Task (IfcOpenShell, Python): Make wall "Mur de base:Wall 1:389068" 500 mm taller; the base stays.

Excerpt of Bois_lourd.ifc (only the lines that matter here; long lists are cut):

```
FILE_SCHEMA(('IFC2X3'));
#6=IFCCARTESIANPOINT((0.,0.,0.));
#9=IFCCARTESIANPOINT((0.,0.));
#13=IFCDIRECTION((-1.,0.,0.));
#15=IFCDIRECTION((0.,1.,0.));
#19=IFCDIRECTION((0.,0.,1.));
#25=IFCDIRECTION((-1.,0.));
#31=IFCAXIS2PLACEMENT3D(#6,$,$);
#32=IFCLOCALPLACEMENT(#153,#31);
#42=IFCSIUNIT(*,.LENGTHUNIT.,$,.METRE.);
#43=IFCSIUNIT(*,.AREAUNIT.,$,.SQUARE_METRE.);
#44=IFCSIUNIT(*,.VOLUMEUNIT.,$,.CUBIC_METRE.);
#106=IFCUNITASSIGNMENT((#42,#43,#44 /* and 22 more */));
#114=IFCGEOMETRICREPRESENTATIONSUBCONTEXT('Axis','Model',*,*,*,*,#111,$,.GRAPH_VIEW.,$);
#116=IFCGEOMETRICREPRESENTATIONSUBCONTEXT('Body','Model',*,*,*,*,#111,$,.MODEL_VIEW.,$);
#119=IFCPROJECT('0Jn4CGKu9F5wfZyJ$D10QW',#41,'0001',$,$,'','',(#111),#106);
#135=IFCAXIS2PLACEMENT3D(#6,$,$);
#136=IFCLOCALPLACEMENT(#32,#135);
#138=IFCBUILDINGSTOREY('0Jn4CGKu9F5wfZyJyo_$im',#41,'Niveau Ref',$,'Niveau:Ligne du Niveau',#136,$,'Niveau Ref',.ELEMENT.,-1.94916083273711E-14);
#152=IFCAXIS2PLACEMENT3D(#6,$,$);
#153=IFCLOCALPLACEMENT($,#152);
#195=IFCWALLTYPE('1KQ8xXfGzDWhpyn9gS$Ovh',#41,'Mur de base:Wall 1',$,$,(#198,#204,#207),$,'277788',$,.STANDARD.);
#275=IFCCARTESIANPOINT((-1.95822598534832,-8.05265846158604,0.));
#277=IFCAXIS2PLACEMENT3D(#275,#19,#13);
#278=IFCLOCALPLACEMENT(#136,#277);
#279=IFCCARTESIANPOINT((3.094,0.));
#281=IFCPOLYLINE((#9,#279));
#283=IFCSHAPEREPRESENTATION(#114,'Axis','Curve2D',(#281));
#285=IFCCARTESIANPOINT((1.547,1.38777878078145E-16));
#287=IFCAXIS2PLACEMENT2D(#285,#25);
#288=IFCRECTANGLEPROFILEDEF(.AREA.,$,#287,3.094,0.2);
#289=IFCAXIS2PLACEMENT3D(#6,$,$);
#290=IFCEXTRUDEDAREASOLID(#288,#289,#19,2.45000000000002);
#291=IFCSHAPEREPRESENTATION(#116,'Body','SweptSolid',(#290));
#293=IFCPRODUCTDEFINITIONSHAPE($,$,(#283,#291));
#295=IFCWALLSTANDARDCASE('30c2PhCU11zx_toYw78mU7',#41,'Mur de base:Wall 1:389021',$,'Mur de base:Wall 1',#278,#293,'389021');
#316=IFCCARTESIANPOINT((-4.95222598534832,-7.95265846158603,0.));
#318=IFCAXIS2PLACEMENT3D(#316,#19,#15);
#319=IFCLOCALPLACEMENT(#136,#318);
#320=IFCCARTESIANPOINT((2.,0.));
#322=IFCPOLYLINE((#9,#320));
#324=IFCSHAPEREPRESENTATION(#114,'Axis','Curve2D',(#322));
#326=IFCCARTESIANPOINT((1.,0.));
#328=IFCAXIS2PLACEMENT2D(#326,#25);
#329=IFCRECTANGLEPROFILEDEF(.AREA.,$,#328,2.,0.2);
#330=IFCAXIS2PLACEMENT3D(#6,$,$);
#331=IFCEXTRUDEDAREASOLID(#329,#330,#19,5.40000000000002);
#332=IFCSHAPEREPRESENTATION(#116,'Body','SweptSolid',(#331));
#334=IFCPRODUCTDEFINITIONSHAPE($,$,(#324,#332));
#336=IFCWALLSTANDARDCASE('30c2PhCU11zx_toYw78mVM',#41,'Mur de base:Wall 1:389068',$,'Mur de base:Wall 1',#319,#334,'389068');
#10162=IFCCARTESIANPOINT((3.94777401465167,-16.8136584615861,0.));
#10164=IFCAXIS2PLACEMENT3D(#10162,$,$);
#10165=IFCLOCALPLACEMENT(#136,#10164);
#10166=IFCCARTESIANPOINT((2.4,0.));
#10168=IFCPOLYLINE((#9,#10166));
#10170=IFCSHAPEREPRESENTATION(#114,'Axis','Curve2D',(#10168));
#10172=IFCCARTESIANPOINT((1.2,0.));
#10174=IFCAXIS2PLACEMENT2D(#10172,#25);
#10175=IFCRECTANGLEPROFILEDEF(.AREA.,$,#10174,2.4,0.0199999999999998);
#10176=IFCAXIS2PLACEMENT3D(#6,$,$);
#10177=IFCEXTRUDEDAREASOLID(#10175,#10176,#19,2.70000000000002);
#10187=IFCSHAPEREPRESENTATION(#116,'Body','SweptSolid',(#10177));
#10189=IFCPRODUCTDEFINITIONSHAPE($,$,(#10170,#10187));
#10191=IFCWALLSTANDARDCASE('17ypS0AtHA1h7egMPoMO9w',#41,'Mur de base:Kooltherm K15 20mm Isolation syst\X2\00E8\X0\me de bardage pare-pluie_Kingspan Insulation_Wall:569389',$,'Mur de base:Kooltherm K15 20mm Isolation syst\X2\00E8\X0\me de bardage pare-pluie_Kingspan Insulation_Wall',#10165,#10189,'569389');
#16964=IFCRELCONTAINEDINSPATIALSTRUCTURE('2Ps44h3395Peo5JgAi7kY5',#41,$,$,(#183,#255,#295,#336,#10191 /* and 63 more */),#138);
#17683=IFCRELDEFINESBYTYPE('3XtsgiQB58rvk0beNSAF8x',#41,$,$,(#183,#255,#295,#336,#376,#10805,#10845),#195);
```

```python
import ifcopenshell
import ifcopenshell.geom
import ifcopenshell.util.representation
import ifcopenshell.util.shape
import ifcopenshell.util.unit

model = ifcopenshell.open("Bois_lourd.ifc")
unit_scale = ifcopenshell.util.unit.calculate_unit_scale(model)
settings = ifcopenshell.geom.settings()


def volume(element):
    """Net volume in cubic metres, openings subtracted."""
    shape = ifcopenshell.geom.create_shape(settings, element)
    return ifcopenshell.util.shape.get_volume(shape.geometry)


wall = model.by_guid("30c2PhCU11zx_toYw78mVM")
before = volume(wall)

body = ifcopenshell.util.representation.get_representation(wall, "Model", "Body")
solid = body.Items[0]
old_height = solid.Depth
solid.Depth += 0.5 / unit_scale
after = volume(wall)

print(f"height {old_height:g} -> {solid.Depth:g}, volume {before:.3f} -> {after:.3f} m3")

model.write("Bois_lourd_edited.ifc")
```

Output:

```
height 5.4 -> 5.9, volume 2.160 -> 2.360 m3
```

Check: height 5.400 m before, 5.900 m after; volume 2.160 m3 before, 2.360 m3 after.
